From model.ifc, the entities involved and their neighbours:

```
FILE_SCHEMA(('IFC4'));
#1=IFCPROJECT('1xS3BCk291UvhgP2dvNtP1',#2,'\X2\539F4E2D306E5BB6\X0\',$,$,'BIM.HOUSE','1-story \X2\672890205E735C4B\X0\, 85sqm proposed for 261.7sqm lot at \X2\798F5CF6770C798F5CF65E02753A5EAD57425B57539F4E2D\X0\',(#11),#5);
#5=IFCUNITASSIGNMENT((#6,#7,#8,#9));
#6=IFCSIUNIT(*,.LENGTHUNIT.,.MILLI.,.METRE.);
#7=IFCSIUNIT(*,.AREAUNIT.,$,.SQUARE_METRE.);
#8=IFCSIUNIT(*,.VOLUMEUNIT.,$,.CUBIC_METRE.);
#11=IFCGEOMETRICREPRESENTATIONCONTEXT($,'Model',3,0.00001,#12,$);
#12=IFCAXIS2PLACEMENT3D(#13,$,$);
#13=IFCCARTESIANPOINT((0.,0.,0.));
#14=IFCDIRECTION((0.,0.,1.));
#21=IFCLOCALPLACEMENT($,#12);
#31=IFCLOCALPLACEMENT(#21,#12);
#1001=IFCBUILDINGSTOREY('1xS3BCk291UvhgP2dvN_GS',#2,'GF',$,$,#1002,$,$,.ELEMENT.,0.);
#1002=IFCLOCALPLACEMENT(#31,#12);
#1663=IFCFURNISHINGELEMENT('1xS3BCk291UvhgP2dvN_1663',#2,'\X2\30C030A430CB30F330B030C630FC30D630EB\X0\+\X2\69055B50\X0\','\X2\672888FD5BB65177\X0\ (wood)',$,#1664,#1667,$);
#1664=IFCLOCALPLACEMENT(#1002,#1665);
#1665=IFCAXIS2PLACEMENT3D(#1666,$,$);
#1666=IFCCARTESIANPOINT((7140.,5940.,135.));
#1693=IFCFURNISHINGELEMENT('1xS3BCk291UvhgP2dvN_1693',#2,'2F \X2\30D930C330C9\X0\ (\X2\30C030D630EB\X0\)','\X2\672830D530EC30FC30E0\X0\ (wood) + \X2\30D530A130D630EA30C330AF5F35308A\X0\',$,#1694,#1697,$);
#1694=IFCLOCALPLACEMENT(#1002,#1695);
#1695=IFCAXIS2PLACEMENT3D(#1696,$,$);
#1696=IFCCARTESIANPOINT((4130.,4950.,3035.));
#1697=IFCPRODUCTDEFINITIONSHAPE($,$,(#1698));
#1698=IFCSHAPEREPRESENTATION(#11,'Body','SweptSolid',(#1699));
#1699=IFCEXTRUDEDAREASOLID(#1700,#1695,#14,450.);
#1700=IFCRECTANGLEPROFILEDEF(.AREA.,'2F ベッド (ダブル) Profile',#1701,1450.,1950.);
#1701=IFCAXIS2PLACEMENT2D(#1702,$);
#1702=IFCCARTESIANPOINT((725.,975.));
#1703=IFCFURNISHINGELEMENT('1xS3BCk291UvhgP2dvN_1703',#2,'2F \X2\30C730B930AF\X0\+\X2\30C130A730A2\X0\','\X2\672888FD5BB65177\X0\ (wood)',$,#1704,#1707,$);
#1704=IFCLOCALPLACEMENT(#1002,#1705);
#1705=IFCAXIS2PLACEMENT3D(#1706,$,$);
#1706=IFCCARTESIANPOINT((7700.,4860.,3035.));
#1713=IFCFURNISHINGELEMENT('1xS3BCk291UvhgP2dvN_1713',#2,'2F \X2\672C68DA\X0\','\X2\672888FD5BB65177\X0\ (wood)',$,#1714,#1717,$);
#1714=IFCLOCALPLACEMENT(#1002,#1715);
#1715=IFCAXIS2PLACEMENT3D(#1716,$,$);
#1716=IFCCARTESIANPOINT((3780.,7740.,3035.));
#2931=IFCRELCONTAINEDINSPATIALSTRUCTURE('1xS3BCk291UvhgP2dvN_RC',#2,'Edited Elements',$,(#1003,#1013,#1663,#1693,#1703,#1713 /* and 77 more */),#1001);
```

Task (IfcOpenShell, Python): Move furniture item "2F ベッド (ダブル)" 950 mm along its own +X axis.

```python
import ifcopenshell
import ifcopenshell.api.geometry
import ifcopenshell.util.placement
import ifcopenshell.util.unit

model = ifcopenshell.open("model.ifc")
unit_scale = ifcopenshell.util.unit.calculate_unit_scale(model)

item = model.by_guid("1xS3BCk291UvhgP2dvN_1693")
matrix = ifcopenshell.util.placement.get_local_placement(item.ObjectPlacement)
matrix[:3, 3] += matrix[:3, 0] * 0.95 / unit_scale
ifcopenshell.api.geometry.edit_object_placement(model, product=item, matrix=matrix, is_si=False)

print(ifcopenshell.util.placement.get_local_placement(item.ObjectPlacement).round(3) + 0.0)

model.write("model_v2.ifc")
```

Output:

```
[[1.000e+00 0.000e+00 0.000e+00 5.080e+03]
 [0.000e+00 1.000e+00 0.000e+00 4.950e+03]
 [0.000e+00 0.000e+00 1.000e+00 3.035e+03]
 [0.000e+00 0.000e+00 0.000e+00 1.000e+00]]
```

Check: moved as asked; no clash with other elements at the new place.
